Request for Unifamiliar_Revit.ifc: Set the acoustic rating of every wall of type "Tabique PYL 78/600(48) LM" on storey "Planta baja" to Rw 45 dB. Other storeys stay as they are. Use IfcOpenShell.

First a look at what the model holds.

```python
import ifcopenshell
import ifcopenshell.util.element

model = ifcopenshell.open("Unifamiliar_Revit.ifc")
print(model.schema)
storey = next(s for s in model.by_type("IfcBuildingStorey") if s.Name == "Planta baja")
walls = [e for e in ifcopenshell.util.element.get_decomposition(storey) if e.is_a("IfcWall")]
seen = {}
for e in walls:
    element_type = ifcopenshell.util.element.get_type(e)
    key = (element_type.Name if element_type != e and element_type else None, ifcopenshell.util.element.get_pset(e, "Pset_WallCommon", "AcousticRating"))
    seen[key] = seen.get(key, 0) + 1
for (name, value), count in sorted(seen.items(), key=str):
    print(count, "x", name, "|", value)
```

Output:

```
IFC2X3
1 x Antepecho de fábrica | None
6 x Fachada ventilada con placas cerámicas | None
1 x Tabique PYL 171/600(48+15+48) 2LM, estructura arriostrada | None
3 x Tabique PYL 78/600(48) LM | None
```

```python
import ifcopenshell
import ifcopenshell.api.pset
import ifcopenshell.util.element

model = ifcopenshell.open("Unifamiliar_Revit.ifc")

storey = next(s for s in model.by_type("IfcBuildingStorey") if s.Name == "Planta baja")
walls = [e for e in ifcopenshell.util.element.get_decomposition(storey) if e.is_a("IfcWall")]

count = 0
for e in walls:
    element_type = ifcopenshell.util.element.get_type(e)
    if element_type in (None, e) or element_type.Name != "Tabique PYL 78/600(48) LM":
        continue
    # add_pset returns the element's existing set when there is one.
    pset = ifcopenshell.api.pset.add_pset(model, product=e, name="Pset_WallCommon")
    ifcopenshell.api.pset.edit_pset(model, pset=pset, properties={"AcousticRating": "Rw 45 dB"})
    count += 1

print(count, "walls updated")

model.write("Unifamiliar_Revit_v2.ifc")
```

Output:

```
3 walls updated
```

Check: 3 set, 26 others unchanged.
